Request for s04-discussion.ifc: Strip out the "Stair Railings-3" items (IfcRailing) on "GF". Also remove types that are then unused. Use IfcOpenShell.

First a look at what the model holds.

```python
import ifcopenshell
import ifcopenshell.util.element

model = ifcopenshell.open("s04-discussion.ifc")
print(model.schema)
storey = next(s for s in model.by_type("IfcBuildingStorey") if s.Name == "GF")
railings = [e for e in ifcopenshell.util.element.get_decomposition(storey) if e.is_a("IfcRailing")]
seen = {}
for e in railings:
    element_type = ifcopenshell.util.element.get_type(e)
    name = element_type.Name if element_type not in (None, e) else None
    seen[name] = seen.get(name, 0) + 1
for name, count in sorted(seen.items(), key=str):
    print(count, "x", name)
```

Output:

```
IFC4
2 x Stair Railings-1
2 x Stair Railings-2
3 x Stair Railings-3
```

```python
import ifcopenshell
import ifcopenshell.api.root
import ifcopenshell.util.element

model = ifcopenshell.open("s04-discussion.ifc")

storey = next(s for s in model.by_type("IfcBuildingStorey") if s.Name == "GF")
railings = [e for e in ifcopenshell.util.element.get_decomposition(storey) if e.is_a("IfcRailing")]
targets = [e for e in railings if (t := ifcopenshell.util.element.get_type(e)) not in (None, e) and t.Name == "Stair Railings-3"]
types = {ifcopenshell.util.element.get_type(e) for e in targets} - {None, *targets}

for e in targets:
    ifcopenshell.api.root.remove_product(model, product=e)
print(len(targets), "removed")

unused = [t for t in types if not ifcopenshell.util.element.get_types(t)]
for t in unused:
    ifcopenshell.api.root.remove_product(model, product=t)
print(len(unused), "unused types removed")

model.write("s04-discussion_updated.ifc")
```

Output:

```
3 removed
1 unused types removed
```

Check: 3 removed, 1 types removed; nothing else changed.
